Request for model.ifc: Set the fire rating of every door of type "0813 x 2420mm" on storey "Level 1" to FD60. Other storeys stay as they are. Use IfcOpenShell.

First a look at what the model holds.

```python
import ifcopenshell
import ifcopenshell.util.element

model = ifcopenshell.open("model.ifc")
print(model.schema)
storey = next(s for s in model.by_type("IfcBuildingStorey") if s.Name == "Level 1")
doors = [e for e in ifcopenshell.util.element.get_decomposition(storey) if e.is_a("IfcDoor")]
seen = {}
for e in doors:
    element_type = ifcopenshell.util.element.get_type(e)
    key = (element_type.Name if element_type != e and element_type else None, ifcopenshell.util.element.get_pset(e, "Pset_DoorCommon", "FireRating"))
    seen[key] = seen.get(key, 0) + 1
for (name, value), count in sorted(seen.items(), key=str):
    print(count, "x", name, "|", value)
```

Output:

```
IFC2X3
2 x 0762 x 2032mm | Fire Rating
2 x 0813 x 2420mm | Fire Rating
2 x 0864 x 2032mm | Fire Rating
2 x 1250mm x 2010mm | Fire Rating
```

```python
import ifcopenshell
import ifcopenshell.api.pset
import ifcopenshell.util.element

model = ifcopenshell.open("model.ifc")

storey = next(s for s in model.by_type("IfcBuildingStorey") if s.Name == "Level 1")
doors = [e for e in ifcopenshell.util.element.get_decomposition(storey) if e.is_a("IfcDoor")]

count = 0
for e in doors:
    element_type = ifcopenshell.util.element.get_type(e)
    if element_type in (None, e) or element_type.Name != "0813 x 2420mm":
        continue
    # add_pset returns the element's existing set when there is one.
    pset = ifcopenshell.api.pset.add_pset(model, product=e, name="Pset_DoorCommon")
    ifcopenshell.api.pset.edit_pset(model, pset=pset, properties={"FireRating": "FD60"})
    count += 1

print(count, "doors updated")

model.write("model_edited.ifc")
```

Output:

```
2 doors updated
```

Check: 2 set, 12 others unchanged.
